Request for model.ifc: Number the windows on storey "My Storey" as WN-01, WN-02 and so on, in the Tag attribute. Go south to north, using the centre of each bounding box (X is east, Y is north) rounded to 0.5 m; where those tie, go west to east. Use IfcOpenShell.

First a look at what the model holds.

```python
import ifcopenshell
import ifcopenshell.util.element
import ifcopenshell.util.placement

model = ifcopenshell.open("model.ifc")
print(model.schema)
storey = next(s for s in model.by_type("IfcBuildingStorey") if s.Name == "My Storey")
windows = [e for e in ifcopenshell.util.element.get_decomposition(storey) if e.is_a("IfcWindow")]
for e in sorted(windows, key=lambda e: e.id()):
    origin = ifcopenshell.util.placement.get_local_placement(e.ObjectPlacement)[:3, 3]
    print(e.id(), e.Tag, e.Name, origin.round(2) + 0.0, sep=" | ")
```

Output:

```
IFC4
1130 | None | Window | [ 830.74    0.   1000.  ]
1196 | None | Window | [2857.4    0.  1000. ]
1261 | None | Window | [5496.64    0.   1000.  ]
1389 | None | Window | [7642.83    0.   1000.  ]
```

```python
import ifcopenshell
import ifcopenshell.geom
import ifcopenshell.util.element
import ifcopenshell.util.shape

model = ifcopenshell.open("model.ifc")
settings = ifcopenshell.geom.settings()
settings.set("use-world-coords", True)


def centre(element):
    shape = ifcopenshell.geom.create_shape(settings, element)
    return ifcopenshell.util.shape.get_bbox_centroid(shape.geometry)


storey = next(s for s in model.by_type("IfcBuildingStorey") if s.Name == "My Storey")
windows = [e for e in ifcopenshell.util.element.get_decomposition(storey) if e.is_a("IfcWindow")]

# Insertion points can sit at a corner or the storey origin, so sort by the geometry (in metres).
centres = {e: centre(e) for e in windows}
windows.sort(key=lambda e: (round(centres[e][1] / 0.5), centres[e][0]))

for i, e in enumerate(windows, start=1):
    number = f"WN-{i:02d}"
    e.Tag = number
    print(e.id(), number)

model.write("model_edited.ifc")
```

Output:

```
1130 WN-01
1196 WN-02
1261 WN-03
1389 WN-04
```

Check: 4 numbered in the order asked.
